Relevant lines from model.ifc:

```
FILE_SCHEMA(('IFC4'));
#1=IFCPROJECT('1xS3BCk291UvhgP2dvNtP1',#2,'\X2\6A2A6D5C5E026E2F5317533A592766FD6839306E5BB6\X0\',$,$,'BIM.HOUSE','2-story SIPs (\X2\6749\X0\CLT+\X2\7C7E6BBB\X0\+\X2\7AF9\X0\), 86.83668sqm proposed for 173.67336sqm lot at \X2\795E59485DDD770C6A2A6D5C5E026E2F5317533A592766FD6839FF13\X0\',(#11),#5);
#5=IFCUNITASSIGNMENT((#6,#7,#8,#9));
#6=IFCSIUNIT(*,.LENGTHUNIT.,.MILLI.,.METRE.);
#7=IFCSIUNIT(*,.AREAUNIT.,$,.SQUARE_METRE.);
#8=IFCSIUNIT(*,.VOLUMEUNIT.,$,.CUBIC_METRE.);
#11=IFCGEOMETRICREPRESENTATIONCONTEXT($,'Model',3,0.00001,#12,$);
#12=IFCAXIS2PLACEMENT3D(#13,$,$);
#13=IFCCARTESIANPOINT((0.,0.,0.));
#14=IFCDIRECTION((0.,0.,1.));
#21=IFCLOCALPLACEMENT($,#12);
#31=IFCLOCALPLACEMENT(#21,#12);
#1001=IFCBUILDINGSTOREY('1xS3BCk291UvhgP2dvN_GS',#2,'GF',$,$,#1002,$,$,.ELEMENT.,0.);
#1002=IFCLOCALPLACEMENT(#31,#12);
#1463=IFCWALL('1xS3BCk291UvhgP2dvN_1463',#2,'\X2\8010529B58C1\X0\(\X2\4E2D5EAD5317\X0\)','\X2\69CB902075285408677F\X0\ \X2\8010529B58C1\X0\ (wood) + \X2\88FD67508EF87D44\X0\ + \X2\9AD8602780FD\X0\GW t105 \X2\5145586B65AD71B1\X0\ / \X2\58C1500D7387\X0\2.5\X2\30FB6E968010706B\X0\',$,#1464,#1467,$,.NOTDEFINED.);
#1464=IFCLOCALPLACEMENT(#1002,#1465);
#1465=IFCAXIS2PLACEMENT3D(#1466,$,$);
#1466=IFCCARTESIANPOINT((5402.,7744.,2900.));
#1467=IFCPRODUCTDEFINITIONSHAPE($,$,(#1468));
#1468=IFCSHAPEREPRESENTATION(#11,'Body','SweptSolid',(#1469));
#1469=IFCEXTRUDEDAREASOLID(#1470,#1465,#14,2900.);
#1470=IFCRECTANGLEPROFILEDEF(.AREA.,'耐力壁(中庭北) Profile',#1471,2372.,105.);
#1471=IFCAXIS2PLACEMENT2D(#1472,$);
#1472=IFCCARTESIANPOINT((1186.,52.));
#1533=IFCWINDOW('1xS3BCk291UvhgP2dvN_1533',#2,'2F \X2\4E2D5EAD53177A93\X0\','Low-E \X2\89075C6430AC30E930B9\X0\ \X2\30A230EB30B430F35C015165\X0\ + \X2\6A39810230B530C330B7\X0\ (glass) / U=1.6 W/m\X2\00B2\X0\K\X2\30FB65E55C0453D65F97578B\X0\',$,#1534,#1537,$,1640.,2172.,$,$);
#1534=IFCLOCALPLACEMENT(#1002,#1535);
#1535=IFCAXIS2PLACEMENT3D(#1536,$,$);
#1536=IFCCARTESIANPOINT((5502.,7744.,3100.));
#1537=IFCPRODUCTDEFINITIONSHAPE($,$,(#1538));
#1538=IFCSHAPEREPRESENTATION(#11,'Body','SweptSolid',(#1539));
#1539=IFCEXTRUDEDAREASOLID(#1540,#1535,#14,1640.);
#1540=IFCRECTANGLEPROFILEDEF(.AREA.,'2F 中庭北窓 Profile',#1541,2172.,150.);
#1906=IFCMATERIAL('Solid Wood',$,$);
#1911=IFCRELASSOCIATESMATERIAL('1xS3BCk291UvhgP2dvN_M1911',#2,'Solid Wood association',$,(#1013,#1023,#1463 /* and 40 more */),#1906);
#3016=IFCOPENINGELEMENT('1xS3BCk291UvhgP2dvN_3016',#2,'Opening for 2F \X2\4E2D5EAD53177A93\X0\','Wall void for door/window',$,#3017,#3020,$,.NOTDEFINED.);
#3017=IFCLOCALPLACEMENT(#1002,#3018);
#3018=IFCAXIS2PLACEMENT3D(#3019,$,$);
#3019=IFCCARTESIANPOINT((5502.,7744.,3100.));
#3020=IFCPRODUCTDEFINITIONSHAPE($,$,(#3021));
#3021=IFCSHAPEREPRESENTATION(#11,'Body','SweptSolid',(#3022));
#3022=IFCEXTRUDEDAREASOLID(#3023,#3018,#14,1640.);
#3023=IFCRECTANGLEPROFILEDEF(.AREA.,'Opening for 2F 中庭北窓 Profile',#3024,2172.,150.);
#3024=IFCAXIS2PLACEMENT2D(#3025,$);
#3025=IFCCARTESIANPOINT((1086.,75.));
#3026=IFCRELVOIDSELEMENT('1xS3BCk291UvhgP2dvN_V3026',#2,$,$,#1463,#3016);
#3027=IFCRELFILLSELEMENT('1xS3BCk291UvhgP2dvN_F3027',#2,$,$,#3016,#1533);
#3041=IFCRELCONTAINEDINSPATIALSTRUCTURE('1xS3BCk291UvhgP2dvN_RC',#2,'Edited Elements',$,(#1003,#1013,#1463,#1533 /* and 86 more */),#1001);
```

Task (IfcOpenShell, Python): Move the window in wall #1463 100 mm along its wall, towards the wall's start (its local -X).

```python
import ifcopenshell
import ifcopenshell.api.geometry
import ifcopenshell.util.placement

model = ifcopenshell.open("model.ifc")

window = model.by_id(1533)
opening = window.FillsVoids[0].RelatingOpeningElement
wall = opening.VoidsElements[0].RelatingBuildingElement

wall_matrix = ifcopenshell.util.placement.get_local_placement(wall.ObjectPlacement)
shift = wall_matrix[:3, 0] * -100.0
before = ifcopenshell.util.placement.get_local_placement(window.ObjectPlacement)[:3, 3].copy()

# The window is not placed relative to its opening, so move both.
for product in (opening, window):
    matrix = ifcopenshell.util.placement.get_local_placement(product.ObjectPlacement)
    matrix[:3, 3] += shift
    ifcopenshell.api.geometry.edit_object_placement(model, product=product, matrix=matrix, is_si=False)

after = ifcopenshell.util.placement.get_local_placement(window.ObjectPlacement)[:3, 3]
print("window moved by", (after - before).round(3) + 0.0)

model.write("model-out.ifc")
```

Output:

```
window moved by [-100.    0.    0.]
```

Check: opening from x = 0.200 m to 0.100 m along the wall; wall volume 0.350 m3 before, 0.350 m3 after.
